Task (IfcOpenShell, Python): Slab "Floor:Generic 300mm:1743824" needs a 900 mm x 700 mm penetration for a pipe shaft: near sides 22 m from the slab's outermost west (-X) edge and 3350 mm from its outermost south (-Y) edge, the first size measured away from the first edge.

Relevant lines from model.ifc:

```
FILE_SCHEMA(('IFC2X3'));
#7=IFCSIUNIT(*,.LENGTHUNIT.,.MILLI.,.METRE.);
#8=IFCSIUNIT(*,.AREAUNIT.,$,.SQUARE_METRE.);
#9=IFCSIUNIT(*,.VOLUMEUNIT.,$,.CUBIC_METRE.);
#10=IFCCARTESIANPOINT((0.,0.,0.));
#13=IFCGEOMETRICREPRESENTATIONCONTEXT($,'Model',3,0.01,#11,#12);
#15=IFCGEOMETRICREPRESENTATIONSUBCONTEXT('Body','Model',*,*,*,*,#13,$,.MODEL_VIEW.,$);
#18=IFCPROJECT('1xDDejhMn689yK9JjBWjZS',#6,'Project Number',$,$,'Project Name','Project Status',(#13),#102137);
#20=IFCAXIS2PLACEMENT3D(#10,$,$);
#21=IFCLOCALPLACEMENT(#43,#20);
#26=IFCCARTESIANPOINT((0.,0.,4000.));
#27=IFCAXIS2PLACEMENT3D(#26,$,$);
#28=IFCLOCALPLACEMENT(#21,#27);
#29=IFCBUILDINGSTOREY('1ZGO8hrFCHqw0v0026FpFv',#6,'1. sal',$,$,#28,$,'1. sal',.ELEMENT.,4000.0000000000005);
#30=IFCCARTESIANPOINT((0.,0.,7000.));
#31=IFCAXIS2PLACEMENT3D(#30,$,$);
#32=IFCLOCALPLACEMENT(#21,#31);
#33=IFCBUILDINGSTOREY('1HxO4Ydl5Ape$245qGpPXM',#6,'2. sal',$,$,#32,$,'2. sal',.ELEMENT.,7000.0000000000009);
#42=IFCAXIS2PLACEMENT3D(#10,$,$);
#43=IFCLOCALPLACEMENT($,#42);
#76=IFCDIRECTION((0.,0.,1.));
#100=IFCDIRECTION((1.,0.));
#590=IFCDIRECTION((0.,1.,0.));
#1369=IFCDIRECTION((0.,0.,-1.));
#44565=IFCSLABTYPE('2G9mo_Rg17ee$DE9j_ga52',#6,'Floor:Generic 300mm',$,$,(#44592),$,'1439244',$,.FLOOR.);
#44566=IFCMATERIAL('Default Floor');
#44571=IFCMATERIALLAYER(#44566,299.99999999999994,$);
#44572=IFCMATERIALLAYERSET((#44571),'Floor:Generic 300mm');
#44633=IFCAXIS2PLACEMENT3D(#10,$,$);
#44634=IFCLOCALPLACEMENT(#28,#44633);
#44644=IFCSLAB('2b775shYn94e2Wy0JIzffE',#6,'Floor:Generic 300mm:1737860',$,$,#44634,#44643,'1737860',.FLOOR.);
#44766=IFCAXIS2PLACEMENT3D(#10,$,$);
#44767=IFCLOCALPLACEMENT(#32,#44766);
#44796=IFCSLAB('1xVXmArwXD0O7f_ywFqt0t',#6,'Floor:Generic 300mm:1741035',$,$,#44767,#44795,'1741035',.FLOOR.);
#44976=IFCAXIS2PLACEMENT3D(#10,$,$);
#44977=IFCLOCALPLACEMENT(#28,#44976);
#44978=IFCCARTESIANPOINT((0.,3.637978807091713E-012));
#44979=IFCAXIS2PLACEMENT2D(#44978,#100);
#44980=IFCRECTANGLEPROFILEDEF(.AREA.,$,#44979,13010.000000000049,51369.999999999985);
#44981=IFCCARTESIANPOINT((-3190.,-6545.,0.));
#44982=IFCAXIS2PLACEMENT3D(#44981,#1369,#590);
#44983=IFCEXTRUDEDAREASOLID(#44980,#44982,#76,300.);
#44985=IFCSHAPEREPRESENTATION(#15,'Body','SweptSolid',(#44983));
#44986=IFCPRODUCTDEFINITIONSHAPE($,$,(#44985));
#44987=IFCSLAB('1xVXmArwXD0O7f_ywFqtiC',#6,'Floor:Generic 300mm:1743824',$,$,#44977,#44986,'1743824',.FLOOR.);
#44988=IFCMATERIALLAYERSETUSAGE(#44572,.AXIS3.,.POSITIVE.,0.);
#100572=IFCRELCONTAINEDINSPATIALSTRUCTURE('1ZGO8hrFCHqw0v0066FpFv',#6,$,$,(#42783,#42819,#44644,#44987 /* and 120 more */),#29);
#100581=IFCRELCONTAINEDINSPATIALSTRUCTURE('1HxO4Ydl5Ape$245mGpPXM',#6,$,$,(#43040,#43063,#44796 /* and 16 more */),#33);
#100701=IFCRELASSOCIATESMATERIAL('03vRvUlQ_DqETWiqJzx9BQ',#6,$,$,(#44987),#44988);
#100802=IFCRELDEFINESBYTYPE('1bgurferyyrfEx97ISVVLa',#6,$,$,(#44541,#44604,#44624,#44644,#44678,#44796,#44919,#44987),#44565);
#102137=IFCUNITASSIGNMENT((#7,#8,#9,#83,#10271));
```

```python
import numpy as np
import ifcopenshell
import ifcopenshell.api.feature
import ifcopenshell.api.geometry
import ifcopenshell.api.root
import ifcopenshell.geom
import ifcopenshell.util.placement
import ifcopenshell.util.representation
import ifcopenshell.util.shape
import ifcopenshell.util.unit

model = ifcopenshell.open("model.ifc")
unit_scale = ifcopenshell.util.unit.calculate_unit_scale(model)
settings = ifcopenshell.geom.settings()


def volume(element):
    """Net volume in cubic metres, openings subtracted."""
    shape = ifcopenshell.geom.create_shape(settings, element)
    return ifcopenshell.util.shape.get_volume(shape.geometry)


slab = model.by_guid("1xVXmArwXD0O7f_ywFqtiC")
before = volume(slab)

# Extent in the slab's own axes, in metres. The edges named are its -X and -Y sides.
slab_shape = ifcopenshell.geom.create_shape(settings, slab)
vertices = ifcopenshell.util.shape.get_vertices(slab_shape.geometry)
x_min, y_min, bottom = vertices.min(axis=0)
top = vertices[:, 2].max()

opening = ifcopenshell.api.root.create_entity(model, ifc_class="IfcOpeningElement", name="Pipe shaft opening")
context = ifcopenshell.util.representation.get_context(model, "Model", "Body", "MODEL_VIEW")
width, depth = 0.9, 0.7
outline = [(0.0, 0.0), (width, 0.0), (width, depth), (0.0, depth), (0.0, 0.0)]
# Overshoot both faces by 50 mm so the cut is clean.
shape = ifcopenshell.api.geometry.add_slab_representation(
    model, context=context, depth=top - bottom + 0.1, polyline=outline
)
ifcopenshell.api.geometry.assign_representation(model, product=opening, representation=shape)

matrix = ifcopenshell.util.placement.get_local_placement(slab.ObjectPlacement)
matrix[:, 3] = matrix @ np.append(np.array([x_min + 22, y_min + 3.35, bottom - 0.05]) / unit_scale, 1.0)
ifcopenshell.api.geometry.edit_object_placement(model, product=opening, matrix=matrix, is_si=False)
ifcopenshell.api.feature.add_feature(model, feature=opening, element=slab)

after = volume(slab)

print(f"slab volume {before:.3f} -> {after:.3f} m3")

model.write("model_edited.ifc")
```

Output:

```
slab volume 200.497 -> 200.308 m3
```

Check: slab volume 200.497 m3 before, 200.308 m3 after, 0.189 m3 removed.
